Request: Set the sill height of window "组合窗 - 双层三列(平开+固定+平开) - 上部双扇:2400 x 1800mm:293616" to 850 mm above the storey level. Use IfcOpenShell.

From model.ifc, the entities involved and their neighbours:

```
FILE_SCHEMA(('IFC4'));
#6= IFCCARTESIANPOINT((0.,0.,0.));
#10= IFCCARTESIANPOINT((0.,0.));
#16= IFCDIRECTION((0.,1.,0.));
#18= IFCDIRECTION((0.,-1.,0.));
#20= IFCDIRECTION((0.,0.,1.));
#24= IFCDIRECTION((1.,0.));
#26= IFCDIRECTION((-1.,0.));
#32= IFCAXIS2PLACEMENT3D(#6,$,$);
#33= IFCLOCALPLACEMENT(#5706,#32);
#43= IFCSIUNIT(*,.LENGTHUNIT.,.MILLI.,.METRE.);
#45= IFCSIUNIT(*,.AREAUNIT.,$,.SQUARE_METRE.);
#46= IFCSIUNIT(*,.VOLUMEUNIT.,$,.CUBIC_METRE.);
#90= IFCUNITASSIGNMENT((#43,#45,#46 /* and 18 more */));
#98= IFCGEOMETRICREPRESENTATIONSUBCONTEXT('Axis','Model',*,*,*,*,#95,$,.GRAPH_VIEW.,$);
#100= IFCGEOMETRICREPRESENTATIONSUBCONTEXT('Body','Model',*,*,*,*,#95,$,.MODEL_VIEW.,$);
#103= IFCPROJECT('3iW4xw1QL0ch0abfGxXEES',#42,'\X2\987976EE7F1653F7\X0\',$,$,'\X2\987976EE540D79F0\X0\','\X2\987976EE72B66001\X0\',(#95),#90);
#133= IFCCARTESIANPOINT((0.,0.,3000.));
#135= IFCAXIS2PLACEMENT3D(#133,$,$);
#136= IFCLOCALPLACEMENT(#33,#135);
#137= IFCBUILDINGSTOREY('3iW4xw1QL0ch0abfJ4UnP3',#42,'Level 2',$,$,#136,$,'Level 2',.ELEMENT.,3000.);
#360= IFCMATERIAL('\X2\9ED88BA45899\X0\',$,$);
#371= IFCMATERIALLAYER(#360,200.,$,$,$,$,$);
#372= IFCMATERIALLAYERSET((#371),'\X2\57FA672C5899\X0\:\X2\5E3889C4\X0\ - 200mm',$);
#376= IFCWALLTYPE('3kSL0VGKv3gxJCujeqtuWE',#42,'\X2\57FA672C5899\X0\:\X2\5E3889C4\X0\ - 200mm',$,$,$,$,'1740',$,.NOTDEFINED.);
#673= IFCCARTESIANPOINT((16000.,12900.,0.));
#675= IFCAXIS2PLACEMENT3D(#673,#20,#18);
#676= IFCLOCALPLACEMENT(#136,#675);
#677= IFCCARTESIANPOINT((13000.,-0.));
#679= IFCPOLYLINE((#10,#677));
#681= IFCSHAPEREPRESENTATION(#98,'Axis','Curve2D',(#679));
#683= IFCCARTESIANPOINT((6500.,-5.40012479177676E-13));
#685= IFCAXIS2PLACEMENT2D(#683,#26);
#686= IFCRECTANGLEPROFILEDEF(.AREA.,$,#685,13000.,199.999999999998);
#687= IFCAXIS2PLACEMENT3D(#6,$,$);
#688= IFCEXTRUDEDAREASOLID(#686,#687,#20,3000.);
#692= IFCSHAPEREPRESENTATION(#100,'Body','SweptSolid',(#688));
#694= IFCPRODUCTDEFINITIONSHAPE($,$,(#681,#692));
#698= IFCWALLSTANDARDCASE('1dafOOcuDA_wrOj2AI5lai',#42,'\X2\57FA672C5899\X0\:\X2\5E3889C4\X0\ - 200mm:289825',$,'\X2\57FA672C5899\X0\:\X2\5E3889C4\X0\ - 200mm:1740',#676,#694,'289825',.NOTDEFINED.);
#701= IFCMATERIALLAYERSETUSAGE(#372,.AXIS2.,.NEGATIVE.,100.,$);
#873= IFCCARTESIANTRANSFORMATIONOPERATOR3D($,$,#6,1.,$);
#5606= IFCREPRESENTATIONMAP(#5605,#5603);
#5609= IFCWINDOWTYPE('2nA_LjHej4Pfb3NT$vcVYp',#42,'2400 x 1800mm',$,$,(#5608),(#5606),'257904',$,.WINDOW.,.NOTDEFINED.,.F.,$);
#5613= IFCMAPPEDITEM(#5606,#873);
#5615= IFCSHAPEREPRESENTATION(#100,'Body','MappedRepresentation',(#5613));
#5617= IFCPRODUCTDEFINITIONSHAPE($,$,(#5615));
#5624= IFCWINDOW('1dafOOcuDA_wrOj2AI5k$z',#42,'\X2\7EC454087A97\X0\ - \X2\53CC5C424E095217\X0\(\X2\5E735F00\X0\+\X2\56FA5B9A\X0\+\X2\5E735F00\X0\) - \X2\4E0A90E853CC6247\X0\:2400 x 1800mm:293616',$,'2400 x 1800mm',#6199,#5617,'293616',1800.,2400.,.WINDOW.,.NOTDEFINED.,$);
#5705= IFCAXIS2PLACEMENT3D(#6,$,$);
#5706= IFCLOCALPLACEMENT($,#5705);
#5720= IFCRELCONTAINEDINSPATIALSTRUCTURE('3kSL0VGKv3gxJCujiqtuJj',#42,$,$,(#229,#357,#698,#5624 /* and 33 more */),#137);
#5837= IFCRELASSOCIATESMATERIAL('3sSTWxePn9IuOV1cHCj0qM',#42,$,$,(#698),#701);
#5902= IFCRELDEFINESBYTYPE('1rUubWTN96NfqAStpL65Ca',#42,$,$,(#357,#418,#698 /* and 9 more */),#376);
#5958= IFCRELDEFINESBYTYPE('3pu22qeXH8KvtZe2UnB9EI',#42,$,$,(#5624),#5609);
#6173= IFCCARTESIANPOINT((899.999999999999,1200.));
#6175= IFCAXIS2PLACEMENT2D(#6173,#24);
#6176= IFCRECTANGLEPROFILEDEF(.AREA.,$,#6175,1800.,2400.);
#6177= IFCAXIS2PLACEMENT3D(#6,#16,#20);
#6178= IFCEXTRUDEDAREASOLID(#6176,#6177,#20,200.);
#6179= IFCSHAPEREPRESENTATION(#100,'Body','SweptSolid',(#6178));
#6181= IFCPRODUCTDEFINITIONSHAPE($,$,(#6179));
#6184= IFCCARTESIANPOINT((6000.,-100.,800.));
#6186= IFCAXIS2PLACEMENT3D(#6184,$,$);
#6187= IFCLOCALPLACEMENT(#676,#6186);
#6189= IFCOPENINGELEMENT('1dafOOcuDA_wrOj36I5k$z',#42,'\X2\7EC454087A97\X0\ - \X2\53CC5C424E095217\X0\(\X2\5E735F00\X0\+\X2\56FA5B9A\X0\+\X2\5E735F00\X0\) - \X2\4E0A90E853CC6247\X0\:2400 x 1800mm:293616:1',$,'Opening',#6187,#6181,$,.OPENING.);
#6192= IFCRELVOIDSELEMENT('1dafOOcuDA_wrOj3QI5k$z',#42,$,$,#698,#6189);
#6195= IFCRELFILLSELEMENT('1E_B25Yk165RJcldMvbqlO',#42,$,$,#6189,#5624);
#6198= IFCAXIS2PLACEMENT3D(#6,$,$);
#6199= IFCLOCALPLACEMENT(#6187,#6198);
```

```python
import numpy as np
import ifcopenshell
import ifcopenshell.api.geometry
import ifcopenshell.geom
import ifcopenshell.util.element
import ifcopenshell.util.placement
import ifcopenshell.util.shape
import ifcopenshell.util.unit

model = ifcopenshell.open("model.ifc")
unit_scale = ifcopenshell.util.unit.calculate_unit_scale(model)

window = model.by_id(5624)
opening = window.FillsVoids[0].RelatingOpeningElement
storey = ifcopenshell.util.element.get_container(window, ifc_class="IfcBuildingStorey")
level = ifcopenshell.util.placement.get_local_placement(storey.ObjectPlacement)[2, 3]

# The opening's origin need not be at the sill, so measure its lowest point.
shape = ifcopenshell.geom.create_shape(ifcopenshell.geom.settings(), opening)
bottom = ifcopenshell.util.shape.get_shape_bottom_elevation(shape, shape.geometry) / unit_scale
dz = level + 850.0 - bottom

shift = np.array([0.0, 0.0, dz])
# The window is placed relative to its opening, so it follows when the opening moves.
matrix = ifcopenshell.util.placement.get_local_placement(opening.ObjectPlacement)
matrix[:3, 3] += shift
ifcopenshell.api.geometry.edit_object_placement(
    model, product=opening, matrix=matrix, is_si=False, should_transform_children=True
)

print(f"moved by {dz * unit_scale:+.3f} m")

model.write("model_rev.ifc")
```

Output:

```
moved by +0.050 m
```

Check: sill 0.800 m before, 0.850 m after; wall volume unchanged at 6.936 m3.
